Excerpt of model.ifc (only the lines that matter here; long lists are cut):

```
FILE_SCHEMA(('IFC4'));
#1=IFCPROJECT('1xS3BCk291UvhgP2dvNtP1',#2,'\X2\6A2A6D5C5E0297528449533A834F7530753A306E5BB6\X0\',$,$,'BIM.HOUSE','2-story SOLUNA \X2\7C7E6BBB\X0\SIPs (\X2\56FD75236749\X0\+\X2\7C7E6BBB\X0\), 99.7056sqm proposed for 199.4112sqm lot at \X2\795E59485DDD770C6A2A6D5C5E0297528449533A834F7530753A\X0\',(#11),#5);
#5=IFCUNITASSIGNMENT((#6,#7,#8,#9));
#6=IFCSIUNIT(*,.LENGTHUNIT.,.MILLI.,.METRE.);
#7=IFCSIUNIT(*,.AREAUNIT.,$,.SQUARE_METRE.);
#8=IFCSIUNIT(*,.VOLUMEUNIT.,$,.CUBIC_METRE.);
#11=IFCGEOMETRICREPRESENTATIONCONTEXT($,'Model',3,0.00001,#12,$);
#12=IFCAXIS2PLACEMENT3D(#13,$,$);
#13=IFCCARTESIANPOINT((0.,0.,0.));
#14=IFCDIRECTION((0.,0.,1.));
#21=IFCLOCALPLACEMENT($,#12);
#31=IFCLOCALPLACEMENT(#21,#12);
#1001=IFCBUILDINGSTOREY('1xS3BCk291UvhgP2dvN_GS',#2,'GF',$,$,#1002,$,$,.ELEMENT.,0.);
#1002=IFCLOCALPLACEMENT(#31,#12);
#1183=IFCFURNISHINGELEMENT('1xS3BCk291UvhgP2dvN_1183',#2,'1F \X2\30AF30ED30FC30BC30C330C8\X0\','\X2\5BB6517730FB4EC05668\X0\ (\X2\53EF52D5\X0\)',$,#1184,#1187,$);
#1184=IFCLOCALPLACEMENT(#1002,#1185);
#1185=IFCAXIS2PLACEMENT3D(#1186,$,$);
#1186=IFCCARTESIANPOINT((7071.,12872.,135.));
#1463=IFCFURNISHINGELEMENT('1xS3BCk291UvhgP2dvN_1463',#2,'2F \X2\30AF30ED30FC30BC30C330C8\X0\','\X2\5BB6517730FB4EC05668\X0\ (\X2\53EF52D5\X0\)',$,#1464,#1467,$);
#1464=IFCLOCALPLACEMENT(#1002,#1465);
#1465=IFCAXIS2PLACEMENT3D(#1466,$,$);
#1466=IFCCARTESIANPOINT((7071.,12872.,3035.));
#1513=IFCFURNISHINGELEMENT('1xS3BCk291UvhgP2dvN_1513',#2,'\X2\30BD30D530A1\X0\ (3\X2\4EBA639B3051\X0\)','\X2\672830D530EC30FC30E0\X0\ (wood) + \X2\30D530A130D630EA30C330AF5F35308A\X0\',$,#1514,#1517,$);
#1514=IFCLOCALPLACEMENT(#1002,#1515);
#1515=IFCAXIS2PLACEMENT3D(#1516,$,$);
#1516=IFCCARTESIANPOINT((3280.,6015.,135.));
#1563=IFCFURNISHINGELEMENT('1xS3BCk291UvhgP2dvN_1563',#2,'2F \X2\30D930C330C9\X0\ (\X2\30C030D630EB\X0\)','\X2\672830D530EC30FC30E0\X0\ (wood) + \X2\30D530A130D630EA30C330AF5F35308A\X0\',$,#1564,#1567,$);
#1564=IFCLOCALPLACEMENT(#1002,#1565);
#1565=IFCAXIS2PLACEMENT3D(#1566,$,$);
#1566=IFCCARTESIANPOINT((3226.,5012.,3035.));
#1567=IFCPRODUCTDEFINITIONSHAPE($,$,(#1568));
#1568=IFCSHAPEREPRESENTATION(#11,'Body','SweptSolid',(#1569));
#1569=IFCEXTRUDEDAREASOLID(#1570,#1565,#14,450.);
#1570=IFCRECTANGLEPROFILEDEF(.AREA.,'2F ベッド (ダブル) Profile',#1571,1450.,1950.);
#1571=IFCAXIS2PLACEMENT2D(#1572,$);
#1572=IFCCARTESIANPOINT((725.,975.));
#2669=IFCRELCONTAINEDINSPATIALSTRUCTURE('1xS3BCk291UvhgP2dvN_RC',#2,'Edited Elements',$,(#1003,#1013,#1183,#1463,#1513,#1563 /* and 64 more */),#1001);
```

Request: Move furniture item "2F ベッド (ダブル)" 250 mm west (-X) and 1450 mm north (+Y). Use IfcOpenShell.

```python
import ifcopenshell
import ifcopenshell.api.geometry
import ifcopenshell.util.placement
import ifcopenshell.util.unit

model = ifcopenshell.open("model.ifc")
unit_scale = ifcopenshell.util.unit.calculate_unit_scale(model)

item = model.by_guid("1xS3BCk291UvhgP2dvN_1563")
matrix = ifcopenshell.util.placement.get_local_placement(item.ObjectPlacement)
matrix[0, 3] -= 0.25 / unit_scale
matrix[1, 3] += 1.45 / unit_scale
ifcopenshell.api.geometry.edit_object_placement(model, product=item, matrix=matrix, is_si=False)

print(ifcopenshell.util.placement.get_local_placement(item.ObjectPlacement).round(3) + 0.0)

model.write("model-out.ifc")
```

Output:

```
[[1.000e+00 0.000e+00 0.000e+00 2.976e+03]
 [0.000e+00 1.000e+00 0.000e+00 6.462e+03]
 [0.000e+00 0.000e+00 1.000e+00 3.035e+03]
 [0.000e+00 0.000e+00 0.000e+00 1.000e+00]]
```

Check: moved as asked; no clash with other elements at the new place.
